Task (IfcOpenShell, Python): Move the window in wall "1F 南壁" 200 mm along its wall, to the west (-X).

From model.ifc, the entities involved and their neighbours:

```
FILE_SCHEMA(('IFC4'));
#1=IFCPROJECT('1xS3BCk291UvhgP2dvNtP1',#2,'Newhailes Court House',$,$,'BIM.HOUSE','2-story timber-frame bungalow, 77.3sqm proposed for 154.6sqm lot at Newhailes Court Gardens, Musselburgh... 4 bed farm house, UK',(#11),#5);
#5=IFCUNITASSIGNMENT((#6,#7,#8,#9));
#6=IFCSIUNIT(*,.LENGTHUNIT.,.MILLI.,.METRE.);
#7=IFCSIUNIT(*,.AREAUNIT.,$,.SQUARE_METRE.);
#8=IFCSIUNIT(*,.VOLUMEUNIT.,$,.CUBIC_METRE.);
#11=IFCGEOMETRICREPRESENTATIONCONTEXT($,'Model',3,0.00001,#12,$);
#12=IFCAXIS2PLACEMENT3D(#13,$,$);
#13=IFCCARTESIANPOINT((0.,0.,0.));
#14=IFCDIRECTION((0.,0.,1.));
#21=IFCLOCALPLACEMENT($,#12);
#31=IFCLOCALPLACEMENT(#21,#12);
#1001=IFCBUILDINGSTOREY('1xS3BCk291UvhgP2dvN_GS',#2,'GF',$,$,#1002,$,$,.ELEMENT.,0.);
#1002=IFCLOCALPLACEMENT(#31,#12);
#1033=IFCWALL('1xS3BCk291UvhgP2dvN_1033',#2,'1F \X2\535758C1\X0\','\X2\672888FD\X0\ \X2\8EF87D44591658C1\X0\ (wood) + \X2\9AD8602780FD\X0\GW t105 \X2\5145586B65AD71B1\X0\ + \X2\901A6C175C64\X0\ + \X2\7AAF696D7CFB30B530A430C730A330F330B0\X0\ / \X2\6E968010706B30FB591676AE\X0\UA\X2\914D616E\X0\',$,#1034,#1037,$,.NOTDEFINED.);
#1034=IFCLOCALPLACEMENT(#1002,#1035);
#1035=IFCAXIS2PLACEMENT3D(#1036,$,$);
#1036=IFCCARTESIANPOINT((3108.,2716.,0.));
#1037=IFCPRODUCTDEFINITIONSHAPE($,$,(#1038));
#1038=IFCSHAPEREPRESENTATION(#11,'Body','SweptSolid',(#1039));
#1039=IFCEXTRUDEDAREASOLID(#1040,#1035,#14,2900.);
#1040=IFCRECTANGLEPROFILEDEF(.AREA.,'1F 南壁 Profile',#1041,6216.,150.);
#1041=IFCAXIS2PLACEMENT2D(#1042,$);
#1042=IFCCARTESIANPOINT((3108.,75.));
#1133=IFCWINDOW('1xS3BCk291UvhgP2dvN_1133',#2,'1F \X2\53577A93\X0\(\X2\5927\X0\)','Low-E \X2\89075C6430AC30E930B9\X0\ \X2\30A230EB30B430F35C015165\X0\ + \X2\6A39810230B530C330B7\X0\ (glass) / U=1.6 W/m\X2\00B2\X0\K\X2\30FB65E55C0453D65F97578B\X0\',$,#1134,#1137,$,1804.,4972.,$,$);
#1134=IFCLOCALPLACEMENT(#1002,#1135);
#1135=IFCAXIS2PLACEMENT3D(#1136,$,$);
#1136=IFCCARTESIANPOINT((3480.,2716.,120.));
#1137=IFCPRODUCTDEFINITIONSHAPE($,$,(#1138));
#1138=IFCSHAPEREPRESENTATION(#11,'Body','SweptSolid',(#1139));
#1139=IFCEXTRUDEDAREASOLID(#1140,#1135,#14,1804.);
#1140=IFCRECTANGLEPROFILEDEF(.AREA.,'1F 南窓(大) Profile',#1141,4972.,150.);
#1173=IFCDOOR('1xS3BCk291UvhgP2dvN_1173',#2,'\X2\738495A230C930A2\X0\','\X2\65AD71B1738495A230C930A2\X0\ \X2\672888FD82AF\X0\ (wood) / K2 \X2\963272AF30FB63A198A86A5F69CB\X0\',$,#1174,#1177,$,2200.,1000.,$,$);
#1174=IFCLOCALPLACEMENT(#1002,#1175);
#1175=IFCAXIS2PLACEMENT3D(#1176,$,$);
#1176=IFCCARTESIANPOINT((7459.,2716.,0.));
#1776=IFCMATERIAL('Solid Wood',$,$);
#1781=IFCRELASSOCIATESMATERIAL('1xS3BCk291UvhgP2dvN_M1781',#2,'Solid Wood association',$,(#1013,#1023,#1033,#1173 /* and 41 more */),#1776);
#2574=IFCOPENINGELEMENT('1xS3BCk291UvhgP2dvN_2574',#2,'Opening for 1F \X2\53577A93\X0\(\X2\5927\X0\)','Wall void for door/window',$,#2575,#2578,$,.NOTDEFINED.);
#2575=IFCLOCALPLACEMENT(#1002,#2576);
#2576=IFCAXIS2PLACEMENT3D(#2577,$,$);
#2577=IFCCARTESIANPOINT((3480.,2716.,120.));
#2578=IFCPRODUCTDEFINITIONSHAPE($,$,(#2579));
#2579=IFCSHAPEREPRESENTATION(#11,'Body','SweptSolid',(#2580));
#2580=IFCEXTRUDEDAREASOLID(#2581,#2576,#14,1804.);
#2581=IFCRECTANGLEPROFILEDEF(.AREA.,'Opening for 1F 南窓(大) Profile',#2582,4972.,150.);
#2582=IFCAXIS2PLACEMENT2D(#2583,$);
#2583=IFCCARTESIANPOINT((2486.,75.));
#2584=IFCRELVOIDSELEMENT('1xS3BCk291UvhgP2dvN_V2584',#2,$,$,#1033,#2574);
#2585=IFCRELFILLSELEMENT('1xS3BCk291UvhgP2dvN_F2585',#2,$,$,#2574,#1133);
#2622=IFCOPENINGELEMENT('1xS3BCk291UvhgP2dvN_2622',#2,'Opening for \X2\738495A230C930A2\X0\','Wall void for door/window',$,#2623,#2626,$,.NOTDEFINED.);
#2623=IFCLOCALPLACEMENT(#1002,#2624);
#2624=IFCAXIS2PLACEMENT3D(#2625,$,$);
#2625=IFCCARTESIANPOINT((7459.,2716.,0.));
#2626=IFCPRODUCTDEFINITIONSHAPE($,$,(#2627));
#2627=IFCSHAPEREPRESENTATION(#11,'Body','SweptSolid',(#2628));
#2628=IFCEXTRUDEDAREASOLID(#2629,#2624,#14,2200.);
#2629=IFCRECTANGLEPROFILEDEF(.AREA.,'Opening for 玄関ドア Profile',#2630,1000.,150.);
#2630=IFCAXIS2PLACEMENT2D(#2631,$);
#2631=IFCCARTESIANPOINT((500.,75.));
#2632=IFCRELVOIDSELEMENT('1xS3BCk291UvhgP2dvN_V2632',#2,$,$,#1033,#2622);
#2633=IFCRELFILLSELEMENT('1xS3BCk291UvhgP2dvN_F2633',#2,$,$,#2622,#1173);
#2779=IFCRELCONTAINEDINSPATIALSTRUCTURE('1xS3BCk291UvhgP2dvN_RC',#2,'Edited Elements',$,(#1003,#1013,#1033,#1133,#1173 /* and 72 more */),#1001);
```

```python
import ifcopenshell
import ifcopenshell.api.geometry
import ifcopenshell.util.placement
import ifcopenshell.util.unit

model = ifcopenshell.open("model.ifc")
unit_scale = ifcopenshell.util.unit.calculate_unit_scale(model)

window = model.by_guid("1xS3BCk291UvhgP2dvN_1133")
opening = window.FillsVoids[0].RelatingOpeningElement
wall = opening.VoidsElements[0].RelatingBuildingElement

wall_matrix = ifcopenshell.util.placement.get_local_placement(wall.ObjectPlacement)
shift = wall_matrix[:3, 0] * -0.2 / unit_scale
before = ifcopenshell.util.placement.get_local_placement(window.ObjectPlacement)[:3, 3].copy()

# The window is not placed relative to its opening, so move both.
for product in (opening, window):
    matrix = ifcopenshell.util.placement.get_local_placement(product.ObjectPlacement)
    matrix[:3, 3] += shift
    ifcopenshell.api.geometry.edit_object_placement(model, product=product, matrix=matrix, is_si=False)

after = ifcopenshell.util.placement.get_local_placement(window.ObjectPlacement)[:3, 3]
print("window moved by", (after - before).round(3) + 0.0)

model.write("model_edited.ifc")
```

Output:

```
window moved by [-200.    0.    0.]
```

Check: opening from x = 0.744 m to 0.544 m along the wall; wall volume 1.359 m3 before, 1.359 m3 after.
